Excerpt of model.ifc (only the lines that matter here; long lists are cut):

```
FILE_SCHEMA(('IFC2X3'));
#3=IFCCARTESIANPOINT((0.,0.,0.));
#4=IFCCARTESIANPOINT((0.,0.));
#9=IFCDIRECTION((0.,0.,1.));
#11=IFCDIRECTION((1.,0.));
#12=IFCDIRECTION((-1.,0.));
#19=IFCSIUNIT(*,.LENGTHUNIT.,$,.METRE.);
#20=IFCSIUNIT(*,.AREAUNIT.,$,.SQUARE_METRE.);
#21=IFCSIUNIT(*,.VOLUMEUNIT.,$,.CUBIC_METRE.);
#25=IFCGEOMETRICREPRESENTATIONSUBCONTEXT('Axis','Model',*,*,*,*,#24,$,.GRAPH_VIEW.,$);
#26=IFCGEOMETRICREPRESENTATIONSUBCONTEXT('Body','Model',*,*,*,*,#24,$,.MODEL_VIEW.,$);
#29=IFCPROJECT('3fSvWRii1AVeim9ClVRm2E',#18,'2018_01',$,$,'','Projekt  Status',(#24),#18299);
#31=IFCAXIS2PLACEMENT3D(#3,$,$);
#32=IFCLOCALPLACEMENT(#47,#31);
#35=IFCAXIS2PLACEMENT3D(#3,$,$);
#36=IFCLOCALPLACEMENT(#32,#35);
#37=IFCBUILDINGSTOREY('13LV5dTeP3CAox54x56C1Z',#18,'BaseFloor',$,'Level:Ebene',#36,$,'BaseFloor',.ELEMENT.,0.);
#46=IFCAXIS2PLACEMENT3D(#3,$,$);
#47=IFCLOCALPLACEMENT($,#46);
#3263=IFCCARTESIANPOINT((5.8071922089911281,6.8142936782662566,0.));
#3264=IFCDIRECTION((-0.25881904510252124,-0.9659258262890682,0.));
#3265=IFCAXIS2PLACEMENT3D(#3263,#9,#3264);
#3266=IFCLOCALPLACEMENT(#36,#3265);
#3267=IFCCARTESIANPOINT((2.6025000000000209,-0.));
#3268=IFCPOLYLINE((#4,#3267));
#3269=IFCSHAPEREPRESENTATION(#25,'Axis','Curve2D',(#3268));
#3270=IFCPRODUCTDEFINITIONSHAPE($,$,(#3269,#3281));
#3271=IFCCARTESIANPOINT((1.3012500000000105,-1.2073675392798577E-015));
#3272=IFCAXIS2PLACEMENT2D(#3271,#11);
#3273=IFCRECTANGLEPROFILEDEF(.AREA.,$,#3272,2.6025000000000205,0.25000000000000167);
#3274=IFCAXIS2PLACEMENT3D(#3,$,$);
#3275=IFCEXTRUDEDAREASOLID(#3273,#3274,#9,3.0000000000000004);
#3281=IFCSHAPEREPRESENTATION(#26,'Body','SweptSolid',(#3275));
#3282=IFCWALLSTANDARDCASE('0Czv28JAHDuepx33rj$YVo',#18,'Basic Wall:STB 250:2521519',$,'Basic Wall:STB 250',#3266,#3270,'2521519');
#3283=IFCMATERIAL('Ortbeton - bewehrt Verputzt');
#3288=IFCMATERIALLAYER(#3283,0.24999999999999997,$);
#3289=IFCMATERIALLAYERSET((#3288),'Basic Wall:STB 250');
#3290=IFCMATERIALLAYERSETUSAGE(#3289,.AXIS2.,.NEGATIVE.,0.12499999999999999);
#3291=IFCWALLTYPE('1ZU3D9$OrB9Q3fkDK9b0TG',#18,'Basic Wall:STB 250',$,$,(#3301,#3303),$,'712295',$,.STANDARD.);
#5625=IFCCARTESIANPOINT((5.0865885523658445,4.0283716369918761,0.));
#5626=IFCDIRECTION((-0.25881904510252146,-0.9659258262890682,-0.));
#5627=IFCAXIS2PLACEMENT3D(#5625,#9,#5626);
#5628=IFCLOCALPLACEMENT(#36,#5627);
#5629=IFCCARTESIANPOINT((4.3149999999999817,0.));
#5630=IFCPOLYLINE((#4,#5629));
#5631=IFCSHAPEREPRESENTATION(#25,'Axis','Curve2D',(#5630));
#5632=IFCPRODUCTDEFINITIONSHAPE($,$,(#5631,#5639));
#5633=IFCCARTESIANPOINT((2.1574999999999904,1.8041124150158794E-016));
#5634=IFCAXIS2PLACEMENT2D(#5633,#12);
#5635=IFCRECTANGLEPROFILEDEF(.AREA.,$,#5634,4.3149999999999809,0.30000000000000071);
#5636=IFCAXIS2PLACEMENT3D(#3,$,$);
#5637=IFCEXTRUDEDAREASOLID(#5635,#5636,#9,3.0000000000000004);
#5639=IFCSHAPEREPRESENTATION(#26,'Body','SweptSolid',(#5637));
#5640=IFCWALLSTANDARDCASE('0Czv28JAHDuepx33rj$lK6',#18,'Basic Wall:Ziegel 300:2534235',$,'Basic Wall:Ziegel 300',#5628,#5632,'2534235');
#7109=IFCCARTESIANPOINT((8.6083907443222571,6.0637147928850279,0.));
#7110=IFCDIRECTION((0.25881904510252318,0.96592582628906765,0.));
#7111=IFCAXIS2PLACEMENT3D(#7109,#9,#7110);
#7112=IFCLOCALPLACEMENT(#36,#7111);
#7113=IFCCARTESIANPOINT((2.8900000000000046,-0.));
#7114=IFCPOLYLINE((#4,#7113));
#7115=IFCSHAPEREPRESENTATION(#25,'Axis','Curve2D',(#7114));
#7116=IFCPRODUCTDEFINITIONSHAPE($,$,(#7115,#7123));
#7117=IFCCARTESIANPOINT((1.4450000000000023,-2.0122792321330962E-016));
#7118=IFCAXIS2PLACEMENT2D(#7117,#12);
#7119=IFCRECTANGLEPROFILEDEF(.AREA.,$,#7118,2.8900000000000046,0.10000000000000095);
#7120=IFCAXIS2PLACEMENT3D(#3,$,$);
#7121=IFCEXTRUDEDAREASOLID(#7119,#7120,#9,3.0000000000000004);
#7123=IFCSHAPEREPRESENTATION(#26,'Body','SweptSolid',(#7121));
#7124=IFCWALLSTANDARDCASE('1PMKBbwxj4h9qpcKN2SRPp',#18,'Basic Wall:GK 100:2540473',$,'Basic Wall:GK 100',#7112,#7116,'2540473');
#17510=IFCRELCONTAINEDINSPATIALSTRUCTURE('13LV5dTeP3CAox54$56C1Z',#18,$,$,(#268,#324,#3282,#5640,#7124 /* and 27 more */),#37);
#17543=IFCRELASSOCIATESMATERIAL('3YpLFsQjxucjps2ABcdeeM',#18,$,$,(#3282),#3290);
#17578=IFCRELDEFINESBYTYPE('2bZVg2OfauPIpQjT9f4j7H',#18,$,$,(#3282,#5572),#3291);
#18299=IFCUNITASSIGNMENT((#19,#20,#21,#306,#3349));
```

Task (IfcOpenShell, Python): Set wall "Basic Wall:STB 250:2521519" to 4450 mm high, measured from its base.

```python
import ifcopenshell
import ifcopenshell.geom
import ifcopenshell.util.representation
import ifcopenshell.util.shape

model = ifcopenshell.open("model.ifc")
settings = ifcopenshell.geom.settings()


def volume(element):
    """Net volume in cubic metres, openings subtracted."""
    shape = ifcopenshell.geom.create_shape(settings, element)
    return ifcopenshell.util.shape.get_volume(shape.geometry)


wall = model.by_id(3282)
before = volume(wall)

body = ifcopenshell.util.representation.get_representation(wall, "Model", "Body")
solid = body.Items[0]
old_height = solid.Depth
solid.Depth = 4.45
after = volume(wall)

print(f"height {old_height:g} -> {solid.Depth:g}, volume {before:.3f} -> {after:.3f} m3")

model.write("model_edited.ifc")
```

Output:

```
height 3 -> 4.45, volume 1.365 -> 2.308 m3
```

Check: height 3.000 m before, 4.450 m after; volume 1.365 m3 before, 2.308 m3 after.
